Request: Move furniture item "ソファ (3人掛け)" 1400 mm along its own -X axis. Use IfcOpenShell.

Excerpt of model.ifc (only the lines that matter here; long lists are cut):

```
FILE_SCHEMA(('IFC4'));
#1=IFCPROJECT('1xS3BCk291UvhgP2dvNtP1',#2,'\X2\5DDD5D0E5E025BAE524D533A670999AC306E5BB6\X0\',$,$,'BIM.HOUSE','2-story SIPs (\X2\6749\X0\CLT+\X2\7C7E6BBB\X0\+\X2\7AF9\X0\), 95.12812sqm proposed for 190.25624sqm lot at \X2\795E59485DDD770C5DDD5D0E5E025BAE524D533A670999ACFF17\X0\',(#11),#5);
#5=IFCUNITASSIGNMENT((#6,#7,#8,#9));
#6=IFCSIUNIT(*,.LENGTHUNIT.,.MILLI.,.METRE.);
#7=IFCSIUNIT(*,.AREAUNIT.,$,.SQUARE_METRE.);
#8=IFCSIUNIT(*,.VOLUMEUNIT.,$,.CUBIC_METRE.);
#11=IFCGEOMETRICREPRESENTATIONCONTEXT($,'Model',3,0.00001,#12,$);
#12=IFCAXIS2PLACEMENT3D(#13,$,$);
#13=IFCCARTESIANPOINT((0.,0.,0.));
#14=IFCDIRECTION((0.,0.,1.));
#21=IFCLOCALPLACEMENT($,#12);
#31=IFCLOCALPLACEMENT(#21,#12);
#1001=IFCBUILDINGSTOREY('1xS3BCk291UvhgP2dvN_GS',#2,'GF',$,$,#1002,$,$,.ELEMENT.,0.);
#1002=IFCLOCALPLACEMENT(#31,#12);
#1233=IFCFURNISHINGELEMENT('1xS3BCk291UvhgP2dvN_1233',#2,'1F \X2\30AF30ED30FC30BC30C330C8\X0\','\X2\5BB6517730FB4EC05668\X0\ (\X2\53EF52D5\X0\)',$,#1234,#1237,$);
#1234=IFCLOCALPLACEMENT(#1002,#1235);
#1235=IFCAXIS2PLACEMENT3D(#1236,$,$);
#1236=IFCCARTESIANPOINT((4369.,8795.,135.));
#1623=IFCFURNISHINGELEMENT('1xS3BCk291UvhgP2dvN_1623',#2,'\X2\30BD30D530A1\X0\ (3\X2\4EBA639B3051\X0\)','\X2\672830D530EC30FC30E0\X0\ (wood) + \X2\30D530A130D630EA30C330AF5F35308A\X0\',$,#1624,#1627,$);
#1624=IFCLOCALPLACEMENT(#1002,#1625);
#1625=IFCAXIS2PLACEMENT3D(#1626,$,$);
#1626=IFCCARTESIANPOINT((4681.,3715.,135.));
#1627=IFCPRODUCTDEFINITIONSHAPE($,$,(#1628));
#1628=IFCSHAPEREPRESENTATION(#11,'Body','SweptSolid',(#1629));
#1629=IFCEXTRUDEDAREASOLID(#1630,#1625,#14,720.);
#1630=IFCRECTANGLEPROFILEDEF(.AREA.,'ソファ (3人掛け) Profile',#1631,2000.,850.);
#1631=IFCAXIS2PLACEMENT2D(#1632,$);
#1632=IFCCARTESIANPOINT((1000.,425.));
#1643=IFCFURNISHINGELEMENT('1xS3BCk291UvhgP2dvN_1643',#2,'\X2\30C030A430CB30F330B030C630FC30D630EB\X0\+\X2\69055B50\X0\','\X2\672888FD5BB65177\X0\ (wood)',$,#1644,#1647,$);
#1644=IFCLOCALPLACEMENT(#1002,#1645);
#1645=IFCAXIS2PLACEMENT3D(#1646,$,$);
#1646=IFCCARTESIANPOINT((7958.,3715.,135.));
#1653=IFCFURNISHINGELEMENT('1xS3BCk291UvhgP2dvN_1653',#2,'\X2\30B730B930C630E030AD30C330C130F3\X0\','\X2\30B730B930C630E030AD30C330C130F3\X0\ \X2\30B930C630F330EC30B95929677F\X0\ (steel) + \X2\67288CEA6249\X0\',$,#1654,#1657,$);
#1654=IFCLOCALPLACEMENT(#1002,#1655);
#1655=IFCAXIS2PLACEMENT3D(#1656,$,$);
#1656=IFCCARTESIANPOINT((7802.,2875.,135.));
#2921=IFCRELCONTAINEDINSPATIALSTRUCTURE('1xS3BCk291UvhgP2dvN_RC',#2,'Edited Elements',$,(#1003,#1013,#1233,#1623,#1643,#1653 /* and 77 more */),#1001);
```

```python
import ifcopenshell
import ifcopenshell.api.geometry
import ifcopenshell.util.placement
import ifcopenshell.util.unit

model = ifcopenshell.open("model.ifc")
unit_scale = ifcopenshell.util.unit.calculate_unit_scale(model)

item = model.by_id(1623)
matrix = ifcopenshell.util.placement.get_local_placement(item.ObjectPlacement)
matrix[:3, 3] -= matrix[:3, 0] * 1.4 / unit_scale
ifcopenshell.api.geometry.edit_object_placement(model, product=item, matrix=matrix, is_si=False)

print(ifcopenshell.util.placement.get_local_placement(item.ObjectPlacement).round(3) + 0.0)

model.write("model_edited.ifc")
```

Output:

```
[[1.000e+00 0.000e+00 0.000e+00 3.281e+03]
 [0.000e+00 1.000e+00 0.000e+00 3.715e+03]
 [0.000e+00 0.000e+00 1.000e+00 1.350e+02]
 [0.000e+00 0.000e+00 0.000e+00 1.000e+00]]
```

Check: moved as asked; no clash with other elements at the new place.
